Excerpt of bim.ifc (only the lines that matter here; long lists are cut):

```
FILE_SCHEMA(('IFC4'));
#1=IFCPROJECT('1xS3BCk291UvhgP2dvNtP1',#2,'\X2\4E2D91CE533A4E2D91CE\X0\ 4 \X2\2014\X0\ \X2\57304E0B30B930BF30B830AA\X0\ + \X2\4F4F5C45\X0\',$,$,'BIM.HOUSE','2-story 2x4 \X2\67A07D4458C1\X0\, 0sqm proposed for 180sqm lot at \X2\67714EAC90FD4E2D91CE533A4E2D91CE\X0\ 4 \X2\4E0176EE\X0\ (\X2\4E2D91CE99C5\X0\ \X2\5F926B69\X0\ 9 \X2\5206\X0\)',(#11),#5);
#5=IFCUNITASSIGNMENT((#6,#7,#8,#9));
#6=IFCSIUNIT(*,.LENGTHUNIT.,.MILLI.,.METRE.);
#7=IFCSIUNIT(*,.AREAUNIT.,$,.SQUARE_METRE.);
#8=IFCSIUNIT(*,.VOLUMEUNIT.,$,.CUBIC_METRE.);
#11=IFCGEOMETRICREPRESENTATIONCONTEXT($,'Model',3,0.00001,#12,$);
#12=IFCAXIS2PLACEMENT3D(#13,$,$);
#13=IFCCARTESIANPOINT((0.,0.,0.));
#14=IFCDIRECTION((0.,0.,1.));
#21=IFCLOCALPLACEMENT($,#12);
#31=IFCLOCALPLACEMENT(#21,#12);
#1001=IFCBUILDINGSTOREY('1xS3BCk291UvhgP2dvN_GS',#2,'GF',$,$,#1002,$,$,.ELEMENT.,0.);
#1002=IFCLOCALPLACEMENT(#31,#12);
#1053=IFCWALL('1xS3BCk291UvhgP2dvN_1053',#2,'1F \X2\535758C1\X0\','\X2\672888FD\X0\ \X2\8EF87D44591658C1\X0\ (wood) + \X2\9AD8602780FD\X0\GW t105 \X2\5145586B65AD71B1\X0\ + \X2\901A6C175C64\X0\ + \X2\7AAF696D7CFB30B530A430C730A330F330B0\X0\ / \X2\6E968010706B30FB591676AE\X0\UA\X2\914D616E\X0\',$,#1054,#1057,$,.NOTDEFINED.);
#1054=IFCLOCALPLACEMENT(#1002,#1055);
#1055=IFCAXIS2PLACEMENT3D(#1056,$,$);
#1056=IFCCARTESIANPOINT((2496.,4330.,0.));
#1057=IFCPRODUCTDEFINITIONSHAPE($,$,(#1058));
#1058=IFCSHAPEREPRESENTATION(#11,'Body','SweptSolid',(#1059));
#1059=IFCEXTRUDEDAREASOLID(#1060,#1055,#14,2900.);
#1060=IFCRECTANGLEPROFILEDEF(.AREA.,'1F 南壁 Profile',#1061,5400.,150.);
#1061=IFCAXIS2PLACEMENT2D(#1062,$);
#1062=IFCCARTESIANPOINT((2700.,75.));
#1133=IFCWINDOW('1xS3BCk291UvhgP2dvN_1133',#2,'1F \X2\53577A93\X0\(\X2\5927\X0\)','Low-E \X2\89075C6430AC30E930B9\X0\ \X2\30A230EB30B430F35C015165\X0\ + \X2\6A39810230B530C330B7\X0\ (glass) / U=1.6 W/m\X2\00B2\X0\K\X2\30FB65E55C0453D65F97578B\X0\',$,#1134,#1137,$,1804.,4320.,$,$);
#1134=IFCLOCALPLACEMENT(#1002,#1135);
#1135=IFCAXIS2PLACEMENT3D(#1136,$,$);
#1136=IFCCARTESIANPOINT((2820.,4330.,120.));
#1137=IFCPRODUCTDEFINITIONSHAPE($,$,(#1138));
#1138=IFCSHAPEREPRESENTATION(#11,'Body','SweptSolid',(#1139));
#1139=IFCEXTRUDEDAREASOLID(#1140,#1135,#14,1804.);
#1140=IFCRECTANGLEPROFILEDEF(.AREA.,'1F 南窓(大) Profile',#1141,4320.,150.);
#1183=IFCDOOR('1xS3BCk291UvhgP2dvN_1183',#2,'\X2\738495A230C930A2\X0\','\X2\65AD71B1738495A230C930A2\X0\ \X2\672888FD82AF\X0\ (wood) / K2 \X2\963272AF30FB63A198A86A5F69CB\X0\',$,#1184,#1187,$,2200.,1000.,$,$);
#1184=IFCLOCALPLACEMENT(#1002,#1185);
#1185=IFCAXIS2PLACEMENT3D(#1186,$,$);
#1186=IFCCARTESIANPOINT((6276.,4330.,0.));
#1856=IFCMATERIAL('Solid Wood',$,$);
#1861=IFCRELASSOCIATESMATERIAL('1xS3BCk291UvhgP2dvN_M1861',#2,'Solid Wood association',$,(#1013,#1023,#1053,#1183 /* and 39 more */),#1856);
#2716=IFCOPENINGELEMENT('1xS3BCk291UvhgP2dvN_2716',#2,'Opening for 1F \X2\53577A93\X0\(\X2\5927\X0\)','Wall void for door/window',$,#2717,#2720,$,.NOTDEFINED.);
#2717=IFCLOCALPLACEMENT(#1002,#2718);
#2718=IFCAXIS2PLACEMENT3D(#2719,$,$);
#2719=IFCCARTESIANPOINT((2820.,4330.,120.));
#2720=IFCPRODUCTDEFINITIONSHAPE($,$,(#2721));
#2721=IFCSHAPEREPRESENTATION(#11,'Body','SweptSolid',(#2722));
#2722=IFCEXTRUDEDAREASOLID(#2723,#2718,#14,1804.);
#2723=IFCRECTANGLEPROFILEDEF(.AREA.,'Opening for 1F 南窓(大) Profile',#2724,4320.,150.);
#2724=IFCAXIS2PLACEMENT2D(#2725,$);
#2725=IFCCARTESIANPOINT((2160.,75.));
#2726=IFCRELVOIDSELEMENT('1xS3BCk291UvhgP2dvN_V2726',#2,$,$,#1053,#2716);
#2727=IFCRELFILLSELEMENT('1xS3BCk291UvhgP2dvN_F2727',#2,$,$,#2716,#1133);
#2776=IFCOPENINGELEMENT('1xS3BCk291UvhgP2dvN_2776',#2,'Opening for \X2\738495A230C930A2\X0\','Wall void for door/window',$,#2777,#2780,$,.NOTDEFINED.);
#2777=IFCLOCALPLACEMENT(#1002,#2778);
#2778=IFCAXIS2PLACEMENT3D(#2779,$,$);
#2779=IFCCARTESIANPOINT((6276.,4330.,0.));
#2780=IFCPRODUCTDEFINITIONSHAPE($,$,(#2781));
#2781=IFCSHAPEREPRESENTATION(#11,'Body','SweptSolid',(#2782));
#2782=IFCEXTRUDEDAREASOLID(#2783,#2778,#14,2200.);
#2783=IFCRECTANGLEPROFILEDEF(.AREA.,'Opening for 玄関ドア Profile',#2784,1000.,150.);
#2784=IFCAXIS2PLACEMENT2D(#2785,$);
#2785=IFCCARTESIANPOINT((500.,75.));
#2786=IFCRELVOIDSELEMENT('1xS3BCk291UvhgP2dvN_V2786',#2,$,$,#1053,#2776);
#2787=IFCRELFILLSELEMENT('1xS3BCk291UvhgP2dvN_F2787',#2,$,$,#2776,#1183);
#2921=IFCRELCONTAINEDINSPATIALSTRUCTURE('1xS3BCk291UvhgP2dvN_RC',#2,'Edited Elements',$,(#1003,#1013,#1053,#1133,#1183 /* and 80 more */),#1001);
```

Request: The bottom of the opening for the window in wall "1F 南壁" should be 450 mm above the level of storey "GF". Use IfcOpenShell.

```python
import numpy as np
import ifcopenshell
import ifcopenshell.api.geometry
import ifcopenshell.geom
import ifcopenshell.util.element
import ifcopenshell.util.placement
import ifcopenshell.util.shape
import ifcopenshell.util.unit

model = ifcopenshell.open("bim.ifc")
unit_scale = ifcopenshell.util.unit.calculate_unit_scale(model)

window = model.by_guid("1xS3BCk291UvhgP2dvN_1133")
opening = window.FillsVoids[0].RelatingOpeningElement
storey = ifcopenshell.util.element.get_container(window, ifc_class="IfcBuildingStorey")
level = ifcopenshell.util.placement.get_local_placement(storey.ObjectPlacement)[2, 3]

# The opening's origin need not be at the sill, so measure its lowest point.
shape = ifcopenshell.geom.create_shape(ifcopenshell.geom.settings(), opening)
bottom = ifcopenshell.util.shape.get_shape_bottom_elevation(shape, shape.geometry) / unit_scale
dz = level + 0.45 / unit_scale - bottom

shift = np.array([0.0, 0.0, dz])
# The window is not placed relative to its opening, so move both.
for product in (opening, window):
    matrix = ifcopenshell.util.placement.get_local_placement(product.ObjectPlacement)
    matrix[:3, 3] += shift
    ifcopenshell.api.geometry.edit_object_placement(model, product=product, matrix=matrix, is_si=False)

print(f"moved by {dz * unit_scale:+.3f} m")

model.write("bim_rev.ifc")
```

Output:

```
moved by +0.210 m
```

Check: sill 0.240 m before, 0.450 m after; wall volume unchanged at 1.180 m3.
